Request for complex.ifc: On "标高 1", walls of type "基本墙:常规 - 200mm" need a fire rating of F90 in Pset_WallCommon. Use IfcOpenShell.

First a look at what the model holds.

```python
import ifcopenshell
import ifcopenshell.util.element

model = ifcopenshell.open("complex.ifc")
print(model.schema)
storey = next(s for s in model.by_type("IfcBuildingStorey") if s.Name == "标高 1")
walls = [e for e in ifcopenshell.util.element.get_decomposition(storey) if e.is_a("IfcWall")]
seen = {}
for e in walls:
    element_type = ifcopenshell.util.element.get_type(e)
    key = (element_type.Name if element_type != e and element_type else None, ifcopenshell.util.element.get_pset(e, "Pset_WallCommon", "FireRating"))
    seen[key] = seen.get(key, 0) + 1
for (name, value), count in sorted(seen.items(), key=str):
    print(count, "x", name, "|", value)
```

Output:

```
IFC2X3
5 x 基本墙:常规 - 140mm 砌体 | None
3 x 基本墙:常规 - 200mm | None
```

```python
import ifcopenshell
import ifcopenshell.api.pset
import ifcopenshell.util.element

model = ifcopenshell.open("complex.ifc")

storey = next(s for s in model.by_type("IfcBuildingStorey") if s.Name == "标高 1")
walls = [e for e in ifcopenshell.util.element.get_decomposition(storey) if e.is_a("IfcWall")]

count = 0
for e in walls:
    element_type = ifcopenshell.util.element.get_type(e)
    if element_type in (None, e) or element_type.Name != "基本墙:常规 - 200mm":
        continue
    # add_pset returns the element's existing set when there is one.
    pset = ifcopenshell.api.pset.add_pset(model, product=e, name="Pset_WallCommon")
    ifcopenshell.api.pset.edit_pset(model, pset=pset, properties={"FireRating": "F90"})
    count += 1

print(count, "walls updated")

model.write("complex_v2.ifc")
```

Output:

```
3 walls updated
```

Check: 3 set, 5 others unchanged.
